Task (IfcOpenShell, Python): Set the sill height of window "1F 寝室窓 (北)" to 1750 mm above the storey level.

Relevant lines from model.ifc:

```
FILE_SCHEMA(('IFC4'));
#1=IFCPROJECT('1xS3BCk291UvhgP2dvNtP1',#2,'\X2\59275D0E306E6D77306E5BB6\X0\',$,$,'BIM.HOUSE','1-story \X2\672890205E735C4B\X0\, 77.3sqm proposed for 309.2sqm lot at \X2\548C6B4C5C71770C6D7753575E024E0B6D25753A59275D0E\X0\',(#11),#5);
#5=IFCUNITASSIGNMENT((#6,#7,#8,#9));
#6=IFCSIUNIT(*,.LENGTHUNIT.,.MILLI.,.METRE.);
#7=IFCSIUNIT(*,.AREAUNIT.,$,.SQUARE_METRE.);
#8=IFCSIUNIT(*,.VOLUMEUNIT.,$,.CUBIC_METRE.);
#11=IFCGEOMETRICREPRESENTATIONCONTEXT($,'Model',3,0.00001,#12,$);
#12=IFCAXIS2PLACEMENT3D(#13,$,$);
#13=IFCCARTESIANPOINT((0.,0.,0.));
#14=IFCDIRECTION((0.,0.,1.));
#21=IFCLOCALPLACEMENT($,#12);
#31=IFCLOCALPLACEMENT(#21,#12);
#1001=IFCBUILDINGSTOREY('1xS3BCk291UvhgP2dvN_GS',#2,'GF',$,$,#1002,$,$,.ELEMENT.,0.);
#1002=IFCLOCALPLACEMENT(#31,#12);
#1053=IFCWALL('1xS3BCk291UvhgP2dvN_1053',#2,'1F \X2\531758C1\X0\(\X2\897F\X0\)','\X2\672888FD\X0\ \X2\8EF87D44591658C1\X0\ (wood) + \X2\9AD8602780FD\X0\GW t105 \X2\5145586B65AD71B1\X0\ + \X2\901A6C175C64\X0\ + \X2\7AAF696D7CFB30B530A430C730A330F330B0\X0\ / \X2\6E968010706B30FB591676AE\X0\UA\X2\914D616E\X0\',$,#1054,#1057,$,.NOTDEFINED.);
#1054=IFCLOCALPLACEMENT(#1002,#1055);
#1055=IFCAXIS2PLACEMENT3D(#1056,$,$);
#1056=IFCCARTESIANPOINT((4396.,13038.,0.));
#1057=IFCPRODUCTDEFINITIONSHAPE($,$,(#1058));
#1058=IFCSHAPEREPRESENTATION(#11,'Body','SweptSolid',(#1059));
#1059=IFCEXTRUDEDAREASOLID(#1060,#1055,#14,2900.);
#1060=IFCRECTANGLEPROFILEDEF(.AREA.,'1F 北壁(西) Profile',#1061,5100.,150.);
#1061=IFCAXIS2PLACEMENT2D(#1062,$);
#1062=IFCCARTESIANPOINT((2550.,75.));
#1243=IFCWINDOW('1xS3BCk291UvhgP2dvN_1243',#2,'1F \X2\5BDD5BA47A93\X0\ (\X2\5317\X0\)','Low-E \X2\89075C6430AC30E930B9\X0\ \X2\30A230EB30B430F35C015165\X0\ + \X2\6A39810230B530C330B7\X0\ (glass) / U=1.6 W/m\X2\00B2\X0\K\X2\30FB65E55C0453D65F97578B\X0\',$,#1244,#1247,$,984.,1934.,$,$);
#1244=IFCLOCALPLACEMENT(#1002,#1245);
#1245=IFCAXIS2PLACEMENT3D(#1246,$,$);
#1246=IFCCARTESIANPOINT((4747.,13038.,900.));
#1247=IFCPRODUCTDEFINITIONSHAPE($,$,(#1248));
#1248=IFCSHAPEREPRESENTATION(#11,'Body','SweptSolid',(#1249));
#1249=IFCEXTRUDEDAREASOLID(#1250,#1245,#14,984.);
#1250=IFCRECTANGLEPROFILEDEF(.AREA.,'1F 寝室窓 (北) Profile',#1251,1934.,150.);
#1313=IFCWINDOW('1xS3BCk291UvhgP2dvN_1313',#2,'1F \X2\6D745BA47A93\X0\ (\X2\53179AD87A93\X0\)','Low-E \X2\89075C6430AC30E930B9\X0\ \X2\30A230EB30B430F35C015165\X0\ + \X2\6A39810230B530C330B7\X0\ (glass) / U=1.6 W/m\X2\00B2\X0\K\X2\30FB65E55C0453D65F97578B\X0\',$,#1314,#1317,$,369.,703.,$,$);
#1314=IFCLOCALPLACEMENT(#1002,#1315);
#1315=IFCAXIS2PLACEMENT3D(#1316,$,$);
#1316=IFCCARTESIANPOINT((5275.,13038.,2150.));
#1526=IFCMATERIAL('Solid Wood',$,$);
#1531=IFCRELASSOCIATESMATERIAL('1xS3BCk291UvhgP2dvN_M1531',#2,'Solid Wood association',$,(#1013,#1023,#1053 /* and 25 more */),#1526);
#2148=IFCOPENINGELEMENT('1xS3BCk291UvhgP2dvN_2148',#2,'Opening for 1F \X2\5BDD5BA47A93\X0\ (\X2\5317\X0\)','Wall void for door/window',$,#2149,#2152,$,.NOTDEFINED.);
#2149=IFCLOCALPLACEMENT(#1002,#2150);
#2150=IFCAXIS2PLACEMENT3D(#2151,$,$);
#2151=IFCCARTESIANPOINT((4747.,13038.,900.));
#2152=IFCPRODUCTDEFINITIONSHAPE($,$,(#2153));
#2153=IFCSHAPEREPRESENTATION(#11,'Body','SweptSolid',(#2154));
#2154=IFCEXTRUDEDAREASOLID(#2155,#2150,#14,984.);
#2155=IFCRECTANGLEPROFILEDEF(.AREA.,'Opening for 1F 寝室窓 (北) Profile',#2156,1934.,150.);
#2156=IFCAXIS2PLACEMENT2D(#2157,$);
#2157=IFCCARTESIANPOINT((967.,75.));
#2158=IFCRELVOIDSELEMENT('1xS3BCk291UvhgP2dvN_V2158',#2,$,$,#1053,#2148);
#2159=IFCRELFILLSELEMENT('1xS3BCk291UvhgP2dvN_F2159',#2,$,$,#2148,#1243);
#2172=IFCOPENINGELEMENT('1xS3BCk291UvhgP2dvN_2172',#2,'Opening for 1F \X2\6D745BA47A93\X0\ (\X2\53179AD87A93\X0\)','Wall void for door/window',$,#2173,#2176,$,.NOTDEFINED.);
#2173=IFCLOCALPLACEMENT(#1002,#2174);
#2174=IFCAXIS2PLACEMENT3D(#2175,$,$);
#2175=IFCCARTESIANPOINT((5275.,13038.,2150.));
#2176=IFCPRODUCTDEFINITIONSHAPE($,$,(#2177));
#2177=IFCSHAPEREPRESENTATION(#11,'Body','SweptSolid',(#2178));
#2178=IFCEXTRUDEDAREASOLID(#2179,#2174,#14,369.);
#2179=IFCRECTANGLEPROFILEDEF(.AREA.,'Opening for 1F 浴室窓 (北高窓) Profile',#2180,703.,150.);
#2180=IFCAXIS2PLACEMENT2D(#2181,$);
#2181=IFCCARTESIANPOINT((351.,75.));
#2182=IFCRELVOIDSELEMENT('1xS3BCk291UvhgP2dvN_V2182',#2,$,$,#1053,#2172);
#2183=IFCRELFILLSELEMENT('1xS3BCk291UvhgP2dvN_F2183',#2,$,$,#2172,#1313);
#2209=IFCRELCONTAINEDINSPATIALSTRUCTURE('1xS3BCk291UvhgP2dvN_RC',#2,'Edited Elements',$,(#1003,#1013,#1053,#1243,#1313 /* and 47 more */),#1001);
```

```python
import numpy as np
import ifcopenshell
import ifcopenshell.api.geometry
import ifcopenshell.geom
import ifcopenshell.util.element
import ifcopenshell.util.placement
import ifcopenshell.util.shape
import ifcopenshell.util.unit

model = ifcopenshell.open("model.ifc")
unit_scale = ifcopenshell.util.unit.calculate_unit_scale(model)

window = model.by_id(1243)
opening = window.FillsVoids[0].RelatingOpeningElement
storey = ifcopenshell.util.element.get_container(window, ifc_class="IfcBuildingStorey")
level = ifcopenshell.util.placement.get_local_placement(storey.ObjectPlacement)[2, 3]

# The opening's origin need not be at the sill, so measure its lowest point.
shape = ifcopenshell.geom.create_shape(ifcopenshell.geom.settings(), opening)
bottom = ifcopenshell.util.shape.get_shape_bottom_elevation(shape, shape.geometry) / unit_scale
dz = level + 1750.0 - bottom

shift = np.array([0.0, 0.0, dz])
# The window is not placed relative to its opening, so move both.
for product in (opening, window):
    matrix = ifcopenshell.util.placement.get_local_placement(product.ObjectPlacement)
    matrix[:3, 3] += shift
    ifcopenshell.api.geometry.edit_object_placement(model, product=product, matrix=matrix, is_si=False)

print(f"moved by {dz * unit_scale:+.3f} m")

model.write("model_rev.ifc")
```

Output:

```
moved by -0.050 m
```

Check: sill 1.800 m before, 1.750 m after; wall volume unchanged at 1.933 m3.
